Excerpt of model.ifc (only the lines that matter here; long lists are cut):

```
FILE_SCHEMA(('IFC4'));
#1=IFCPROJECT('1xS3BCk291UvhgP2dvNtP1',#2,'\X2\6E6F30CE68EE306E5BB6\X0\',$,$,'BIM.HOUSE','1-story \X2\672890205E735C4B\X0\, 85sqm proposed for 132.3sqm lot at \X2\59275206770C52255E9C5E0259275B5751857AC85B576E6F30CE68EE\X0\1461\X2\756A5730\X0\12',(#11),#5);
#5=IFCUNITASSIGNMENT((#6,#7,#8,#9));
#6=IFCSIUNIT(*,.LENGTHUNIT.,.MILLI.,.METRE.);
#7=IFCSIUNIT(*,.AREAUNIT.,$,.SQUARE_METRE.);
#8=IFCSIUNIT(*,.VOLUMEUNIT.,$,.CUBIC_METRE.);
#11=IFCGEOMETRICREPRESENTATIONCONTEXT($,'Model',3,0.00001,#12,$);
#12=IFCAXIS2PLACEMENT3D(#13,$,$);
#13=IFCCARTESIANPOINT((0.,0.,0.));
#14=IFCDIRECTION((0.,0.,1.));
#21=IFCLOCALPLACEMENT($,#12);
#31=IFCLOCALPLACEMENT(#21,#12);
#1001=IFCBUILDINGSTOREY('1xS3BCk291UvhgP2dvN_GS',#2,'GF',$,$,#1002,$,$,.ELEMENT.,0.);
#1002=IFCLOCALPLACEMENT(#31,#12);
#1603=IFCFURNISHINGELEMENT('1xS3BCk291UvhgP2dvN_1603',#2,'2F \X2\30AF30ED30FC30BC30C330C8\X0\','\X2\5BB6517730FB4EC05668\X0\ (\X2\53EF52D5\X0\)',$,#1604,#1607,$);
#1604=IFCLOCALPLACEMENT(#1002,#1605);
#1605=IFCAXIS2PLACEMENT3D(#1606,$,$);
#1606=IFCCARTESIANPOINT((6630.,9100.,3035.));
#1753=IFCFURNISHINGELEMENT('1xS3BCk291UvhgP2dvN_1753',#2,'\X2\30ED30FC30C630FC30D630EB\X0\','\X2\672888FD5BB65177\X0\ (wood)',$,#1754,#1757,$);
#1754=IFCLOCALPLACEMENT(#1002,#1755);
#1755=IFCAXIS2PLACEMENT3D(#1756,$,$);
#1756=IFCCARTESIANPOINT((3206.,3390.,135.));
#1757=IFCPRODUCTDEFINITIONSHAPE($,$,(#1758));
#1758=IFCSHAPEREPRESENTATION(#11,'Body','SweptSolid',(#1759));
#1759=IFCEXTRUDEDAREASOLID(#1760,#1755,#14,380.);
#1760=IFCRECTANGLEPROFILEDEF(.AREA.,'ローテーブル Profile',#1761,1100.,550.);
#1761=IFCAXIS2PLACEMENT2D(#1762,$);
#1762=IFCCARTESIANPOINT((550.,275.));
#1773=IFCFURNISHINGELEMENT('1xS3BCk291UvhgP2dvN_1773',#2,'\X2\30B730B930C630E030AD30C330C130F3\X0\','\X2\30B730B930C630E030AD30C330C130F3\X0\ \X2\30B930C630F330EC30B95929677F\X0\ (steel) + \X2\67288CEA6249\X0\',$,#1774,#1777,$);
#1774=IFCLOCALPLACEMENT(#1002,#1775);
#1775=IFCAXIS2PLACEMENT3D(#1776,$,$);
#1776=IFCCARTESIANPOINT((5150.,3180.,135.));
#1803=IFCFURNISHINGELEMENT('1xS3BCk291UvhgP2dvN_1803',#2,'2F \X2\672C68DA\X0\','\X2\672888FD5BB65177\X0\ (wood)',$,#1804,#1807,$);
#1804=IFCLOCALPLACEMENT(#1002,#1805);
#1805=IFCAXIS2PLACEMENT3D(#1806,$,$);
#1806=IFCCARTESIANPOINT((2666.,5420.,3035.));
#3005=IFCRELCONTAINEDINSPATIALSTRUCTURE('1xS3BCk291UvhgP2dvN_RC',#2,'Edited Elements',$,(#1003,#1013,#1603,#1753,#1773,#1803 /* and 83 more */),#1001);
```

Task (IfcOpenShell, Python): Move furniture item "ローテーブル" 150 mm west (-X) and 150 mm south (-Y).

```python
import ifcopenshell
import ifcopenshell.api.geometry
import ifcopenshell.util.placement
import ifcopenshell.util.unit

model = ifcopenshell.open("model.ifc")
unit_scale = ifcopenshell.util.unit.calculate_unit_scale(model)

item = model.by_guid("1xS3BCk291UvhgP2dvN_1753")
matrix = ifcopenshell.util.placement.get_local_placement(item.ObjectPlacement)
matrix[0, 3] -= 0.15 / unit_scale
matrix[1, 3] -= 0.15 / unit_scale
ifcopenshell.api.geometry.edit_object_placement(model, product=item, matrix=matrix, is_si=False)

print(ifcopenshell.util.placement.get_local_placement(item.ObjectPlacement).round(3) + 0.0)

model.write("model_v2.ifc")
```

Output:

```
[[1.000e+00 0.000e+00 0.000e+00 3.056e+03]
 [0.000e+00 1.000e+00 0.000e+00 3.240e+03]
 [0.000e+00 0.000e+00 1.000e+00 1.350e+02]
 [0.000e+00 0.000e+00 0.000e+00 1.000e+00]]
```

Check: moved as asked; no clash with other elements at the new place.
